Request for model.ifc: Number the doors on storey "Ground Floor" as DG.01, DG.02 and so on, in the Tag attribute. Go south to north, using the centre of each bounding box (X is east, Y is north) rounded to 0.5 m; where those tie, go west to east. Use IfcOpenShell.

First a look at what the model holds.

```python
import ifcopenshell
import ifcopenshell.util.element
import ifcopenshell.util.placement

model = ifcopenshell.open("model.ifc")
print(model.schema)
storey = next(s for s in model.by_type("IfcBuildingStorey") if s.Name == "Ground Floor")
doors = [e for e in ifcopenshell.util.element.get_decomposition(storey) if e.is_a("IfcDoor")]
for e in sorted(doors, key=lambda e: e.id()):
    origin = ifcopenshell.util.placement.get_local_placement(e.ObjectPlacement)[:3, 3]
    print(e.id(), e.Tag, e.Name, origin.round(2) + 0.0, sep=" | ")
```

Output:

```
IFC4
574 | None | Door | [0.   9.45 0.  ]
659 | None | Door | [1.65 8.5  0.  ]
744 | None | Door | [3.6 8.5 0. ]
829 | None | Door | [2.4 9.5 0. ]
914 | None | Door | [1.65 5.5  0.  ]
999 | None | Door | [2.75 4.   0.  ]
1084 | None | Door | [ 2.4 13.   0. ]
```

```python
import ifcopenshell
import ifcopenshell.geom
import ifcopenshell.util.element
import ifcopenshell.util.shape

model = ifcopenshell.open("model.ifc")
settings = ifcopenshell.geom.settings()
settings.set("use-world-coords", True)


def centre(element):
    shape = ifcopenshell.geom.create_shape(settings, element)
    return ifcopenshell.util.shape.get_bbox_centroid(shape.geometry)


storey = next(s for s in model.by_type("IfcBuildingStorey") if s.Name == "Ground Floor")
doors = [e for e in ifcopenshell.util.element.get_decomposition(storey) if e.is_a("IfcDoor")]

# Insertion points can sit at a corner or the storey origin, so sort by the geometry (in metres).
centres = {e: centre(e) for e in doors}
doors.sort(key=lambda e: (round(centres[e][1] / 0.5), centres[e][0]))

for i, e in enumerate(doors, start=1):
    number = f"DG.{i:02d}"
    e.Tag = number
    print(e.id(), number)

model.write("model_v2.ifc")
```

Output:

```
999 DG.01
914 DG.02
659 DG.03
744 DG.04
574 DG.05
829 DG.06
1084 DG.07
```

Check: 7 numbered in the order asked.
